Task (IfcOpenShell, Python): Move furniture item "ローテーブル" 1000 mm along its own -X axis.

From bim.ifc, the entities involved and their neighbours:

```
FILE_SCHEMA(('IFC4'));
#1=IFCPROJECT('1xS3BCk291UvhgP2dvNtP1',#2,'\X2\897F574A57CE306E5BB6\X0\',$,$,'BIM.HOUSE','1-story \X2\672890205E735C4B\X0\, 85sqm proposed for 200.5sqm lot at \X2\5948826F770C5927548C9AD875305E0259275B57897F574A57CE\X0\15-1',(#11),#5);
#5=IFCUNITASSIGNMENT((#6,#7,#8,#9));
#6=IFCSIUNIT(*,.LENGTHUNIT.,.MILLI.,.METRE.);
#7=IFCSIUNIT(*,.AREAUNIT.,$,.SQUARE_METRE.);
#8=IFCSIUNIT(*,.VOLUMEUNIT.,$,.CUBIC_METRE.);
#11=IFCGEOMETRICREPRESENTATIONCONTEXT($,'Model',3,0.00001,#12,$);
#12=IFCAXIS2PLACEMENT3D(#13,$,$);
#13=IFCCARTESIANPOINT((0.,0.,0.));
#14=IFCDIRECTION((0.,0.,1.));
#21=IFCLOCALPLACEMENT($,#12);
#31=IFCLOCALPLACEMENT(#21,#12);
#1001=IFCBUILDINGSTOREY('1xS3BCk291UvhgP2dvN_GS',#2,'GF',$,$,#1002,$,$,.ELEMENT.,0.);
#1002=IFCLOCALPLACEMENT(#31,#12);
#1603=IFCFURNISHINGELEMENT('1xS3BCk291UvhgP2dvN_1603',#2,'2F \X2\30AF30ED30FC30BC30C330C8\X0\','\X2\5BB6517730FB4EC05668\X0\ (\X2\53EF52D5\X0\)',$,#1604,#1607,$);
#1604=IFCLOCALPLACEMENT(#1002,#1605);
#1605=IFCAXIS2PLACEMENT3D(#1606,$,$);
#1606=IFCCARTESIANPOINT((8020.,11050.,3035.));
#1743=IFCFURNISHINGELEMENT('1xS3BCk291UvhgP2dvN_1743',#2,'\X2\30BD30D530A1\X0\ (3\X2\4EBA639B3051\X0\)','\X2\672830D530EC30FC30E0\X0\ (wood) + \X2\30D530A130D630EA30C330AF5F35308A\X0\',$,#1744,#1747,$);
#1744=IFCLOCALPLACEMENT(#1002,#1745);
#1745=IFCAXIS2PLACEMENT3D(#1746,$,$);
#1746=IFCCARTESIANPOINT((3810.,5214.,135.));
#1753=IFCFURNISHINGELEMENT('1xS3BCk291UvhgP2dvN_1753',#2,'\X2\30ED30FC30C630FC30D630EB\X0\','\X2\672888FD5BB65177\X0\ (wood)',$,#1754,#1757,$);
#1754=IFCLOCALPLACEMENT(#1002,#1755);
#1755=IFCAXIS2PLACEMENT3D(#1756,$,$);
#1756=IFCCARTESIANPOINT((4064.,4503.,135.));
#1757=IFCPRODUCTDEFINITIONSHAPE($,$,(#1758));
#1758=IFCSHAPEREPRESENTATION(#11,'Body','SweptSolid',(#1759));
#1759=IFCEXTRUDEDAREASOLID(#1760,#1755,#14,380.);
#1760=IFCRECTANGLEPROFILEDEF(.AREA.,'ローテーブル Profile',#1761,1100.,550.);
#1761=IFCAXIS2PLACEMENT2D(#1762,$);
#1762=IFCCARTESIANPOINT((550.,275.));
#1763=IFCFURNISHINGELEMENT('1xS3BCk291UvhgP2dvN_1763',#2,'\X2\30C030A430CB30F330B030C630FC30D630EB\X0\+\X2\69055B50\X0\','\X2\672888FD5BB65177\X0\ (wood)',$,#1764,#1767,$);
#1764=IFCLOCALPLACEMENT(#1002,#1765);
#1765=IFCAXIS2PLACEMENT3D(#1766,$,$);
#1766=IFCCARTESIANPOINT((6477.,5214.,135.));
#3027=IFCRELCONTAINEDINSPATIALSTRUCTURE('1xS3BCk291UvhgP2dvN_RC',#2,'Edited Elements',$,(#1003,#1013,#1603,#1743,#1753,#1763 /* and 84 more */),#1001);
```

```python
import ifcopenshell
import ifcopenshell.api.geometry
import ifcopenshell.util.placement
import ifcopenshell.util.unit

model = ifcopenshell.open("bim.ifc")
unit_scale = ifcopenshell.util.unit.calculate_unit_scale(model)

item = model.by_guid("1xS3BCk291UvhgP2dvN_1753")
matrix = ifcopenshell.util.placement.get_local_placement(item.ObjectPlacement)
matrix[:3, 3] -= matrix[:3, 0] * 1 / unit_scale
ifcopenshell.api.geometry.edit_object_placement(model, product=item, matrix=matrix, is_si=False)

print(ifcopenshell.util.placement.get_local_placement(item.ObjectPlacement).round(3) + 0.0)

model.write("bim_updated.ifc")
```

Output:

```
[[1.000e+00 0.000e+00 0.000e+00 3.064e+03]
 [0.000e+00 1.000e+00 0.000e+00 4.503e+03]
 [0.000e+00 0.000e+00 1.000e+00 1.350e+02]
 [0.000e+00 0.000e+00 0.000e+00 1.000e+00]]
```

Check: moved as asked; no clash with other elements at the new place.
